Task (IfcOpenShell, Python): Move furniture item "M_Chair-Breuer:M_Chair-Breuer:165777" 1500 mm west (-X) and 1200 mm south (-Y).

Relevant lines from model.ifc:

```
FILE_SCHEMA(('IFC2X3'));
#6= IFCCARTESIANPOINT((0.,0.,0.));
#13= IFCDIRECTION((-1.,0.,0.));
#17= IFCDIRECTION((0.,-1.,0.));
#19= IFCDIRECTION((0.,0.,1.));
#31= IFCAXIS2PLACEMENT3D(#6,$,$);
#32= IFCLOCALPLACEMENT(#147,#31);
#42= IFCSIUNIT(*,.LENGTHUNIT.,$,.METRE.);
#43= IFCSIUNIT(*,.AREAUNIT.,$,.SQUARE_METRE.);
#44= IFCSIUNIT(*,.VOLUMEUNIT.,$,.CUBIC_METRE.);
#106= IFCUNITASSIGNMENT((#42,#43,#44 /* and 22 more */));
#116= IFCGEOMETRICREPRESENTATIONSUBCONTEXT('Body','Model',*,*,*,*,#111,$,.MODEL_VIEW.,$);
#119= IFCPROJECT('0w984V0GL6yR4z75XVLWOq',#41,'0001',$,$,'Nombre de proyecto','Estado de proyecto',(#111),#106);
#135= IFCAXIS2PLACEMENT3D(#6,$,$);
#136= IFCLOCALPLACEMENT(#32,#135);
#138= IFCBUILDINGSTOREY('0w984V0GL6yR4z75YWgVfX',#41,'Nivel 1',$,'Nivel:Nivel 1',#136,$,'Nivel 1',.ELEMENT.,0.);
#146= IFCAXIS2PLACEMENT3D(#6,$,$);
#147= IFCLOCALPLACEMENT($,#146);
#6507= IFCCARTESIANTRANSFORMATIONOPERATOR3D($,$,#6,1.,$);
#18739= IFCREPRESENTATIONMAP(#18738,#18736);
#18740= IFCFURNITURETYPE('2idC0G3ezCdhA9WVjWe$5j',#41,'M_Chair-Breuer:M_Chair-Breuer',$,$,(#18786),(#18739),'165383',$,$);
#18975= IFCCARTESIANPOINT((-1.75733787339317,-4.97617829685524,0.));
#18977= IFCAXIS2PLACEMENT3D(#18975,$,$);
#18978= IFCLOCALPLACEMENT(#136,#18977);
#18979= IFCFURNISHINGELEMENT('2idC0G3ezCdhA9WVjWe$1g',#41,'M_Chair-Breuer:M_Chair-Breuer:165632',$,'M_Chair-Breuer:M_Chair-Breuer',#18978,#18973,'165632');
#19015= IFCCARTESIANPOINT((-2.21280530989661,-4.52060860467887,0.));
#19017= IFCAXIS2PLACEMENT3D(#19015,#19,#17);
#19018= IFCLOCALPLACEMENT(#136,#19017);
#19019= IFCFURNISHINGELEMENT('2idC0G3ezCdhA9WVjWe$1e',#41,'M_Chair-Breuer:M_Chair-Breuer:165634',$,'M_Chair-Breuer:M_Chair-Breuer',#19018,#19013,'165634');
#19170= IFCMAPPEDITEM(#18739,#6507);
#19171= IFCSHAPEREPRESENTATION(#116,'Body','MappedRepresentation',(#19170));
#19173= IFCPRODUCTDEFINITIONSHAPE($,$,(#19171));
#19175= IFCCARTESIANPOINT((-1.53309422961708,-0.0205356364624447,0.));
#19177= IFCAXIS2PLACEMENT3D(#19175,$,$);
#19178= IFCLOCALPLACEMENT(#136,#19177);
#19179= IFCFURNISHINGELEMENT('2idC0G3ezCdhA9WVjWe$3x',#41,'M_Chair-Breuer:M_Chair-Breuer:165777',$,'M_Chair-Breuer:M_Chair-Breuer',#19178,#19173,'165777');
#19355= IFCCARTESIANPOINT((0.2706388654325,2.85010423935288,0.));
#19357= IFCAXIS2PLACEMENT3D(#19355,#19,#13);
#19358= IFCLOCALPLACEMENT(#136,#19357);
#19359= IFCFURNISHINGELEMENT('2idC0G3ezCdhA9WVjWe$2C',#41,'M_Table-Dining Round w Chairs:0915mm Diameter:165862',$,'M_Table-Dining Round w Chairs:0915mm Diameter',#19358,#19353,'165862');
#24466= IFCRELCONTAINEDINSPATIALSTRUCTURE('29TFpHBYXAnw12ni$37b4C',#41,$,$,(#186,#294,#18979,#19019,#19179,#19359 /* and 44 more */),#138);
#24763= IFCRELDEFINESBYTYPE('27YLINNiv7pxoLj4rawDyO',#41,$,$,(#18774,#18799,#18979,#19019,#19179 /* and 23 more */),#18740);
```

```python
import ifcopenshell
import ifcopenshell.api.geometry
import ifcopenshell.util.placement
import ifcopenshell.util.unit

model = ifcopenshell.open("model.ifc")
unit_scale = ifcopenshell.util.unit.calculate_unit_scale(model)

item = model.by_guid("2idC0G3ezCdhA9WVjWe$3x")
matrix = ifcopenshell.util.placement.get_local_placement(item.ObjectPlacement)
matrix[0, 3] -= 1.5 / unit_scale
matrix[1, 3] -= 1.2 / unit_scale
ifcopenshell.api.geometry.edit_object_placement(model, product=item, matrix=matrix, is_si=False)

print(ifcopenshell.util.placement.get_local_placement(item.ObjectPlacement).round(3) + 0.0)

model.write("model_v2.ifc")
```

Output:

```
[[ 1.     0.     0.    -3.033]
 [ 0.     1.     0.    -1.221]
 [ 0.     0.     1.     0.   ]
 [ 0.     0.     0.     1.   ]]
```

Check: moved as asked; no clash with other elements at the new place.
